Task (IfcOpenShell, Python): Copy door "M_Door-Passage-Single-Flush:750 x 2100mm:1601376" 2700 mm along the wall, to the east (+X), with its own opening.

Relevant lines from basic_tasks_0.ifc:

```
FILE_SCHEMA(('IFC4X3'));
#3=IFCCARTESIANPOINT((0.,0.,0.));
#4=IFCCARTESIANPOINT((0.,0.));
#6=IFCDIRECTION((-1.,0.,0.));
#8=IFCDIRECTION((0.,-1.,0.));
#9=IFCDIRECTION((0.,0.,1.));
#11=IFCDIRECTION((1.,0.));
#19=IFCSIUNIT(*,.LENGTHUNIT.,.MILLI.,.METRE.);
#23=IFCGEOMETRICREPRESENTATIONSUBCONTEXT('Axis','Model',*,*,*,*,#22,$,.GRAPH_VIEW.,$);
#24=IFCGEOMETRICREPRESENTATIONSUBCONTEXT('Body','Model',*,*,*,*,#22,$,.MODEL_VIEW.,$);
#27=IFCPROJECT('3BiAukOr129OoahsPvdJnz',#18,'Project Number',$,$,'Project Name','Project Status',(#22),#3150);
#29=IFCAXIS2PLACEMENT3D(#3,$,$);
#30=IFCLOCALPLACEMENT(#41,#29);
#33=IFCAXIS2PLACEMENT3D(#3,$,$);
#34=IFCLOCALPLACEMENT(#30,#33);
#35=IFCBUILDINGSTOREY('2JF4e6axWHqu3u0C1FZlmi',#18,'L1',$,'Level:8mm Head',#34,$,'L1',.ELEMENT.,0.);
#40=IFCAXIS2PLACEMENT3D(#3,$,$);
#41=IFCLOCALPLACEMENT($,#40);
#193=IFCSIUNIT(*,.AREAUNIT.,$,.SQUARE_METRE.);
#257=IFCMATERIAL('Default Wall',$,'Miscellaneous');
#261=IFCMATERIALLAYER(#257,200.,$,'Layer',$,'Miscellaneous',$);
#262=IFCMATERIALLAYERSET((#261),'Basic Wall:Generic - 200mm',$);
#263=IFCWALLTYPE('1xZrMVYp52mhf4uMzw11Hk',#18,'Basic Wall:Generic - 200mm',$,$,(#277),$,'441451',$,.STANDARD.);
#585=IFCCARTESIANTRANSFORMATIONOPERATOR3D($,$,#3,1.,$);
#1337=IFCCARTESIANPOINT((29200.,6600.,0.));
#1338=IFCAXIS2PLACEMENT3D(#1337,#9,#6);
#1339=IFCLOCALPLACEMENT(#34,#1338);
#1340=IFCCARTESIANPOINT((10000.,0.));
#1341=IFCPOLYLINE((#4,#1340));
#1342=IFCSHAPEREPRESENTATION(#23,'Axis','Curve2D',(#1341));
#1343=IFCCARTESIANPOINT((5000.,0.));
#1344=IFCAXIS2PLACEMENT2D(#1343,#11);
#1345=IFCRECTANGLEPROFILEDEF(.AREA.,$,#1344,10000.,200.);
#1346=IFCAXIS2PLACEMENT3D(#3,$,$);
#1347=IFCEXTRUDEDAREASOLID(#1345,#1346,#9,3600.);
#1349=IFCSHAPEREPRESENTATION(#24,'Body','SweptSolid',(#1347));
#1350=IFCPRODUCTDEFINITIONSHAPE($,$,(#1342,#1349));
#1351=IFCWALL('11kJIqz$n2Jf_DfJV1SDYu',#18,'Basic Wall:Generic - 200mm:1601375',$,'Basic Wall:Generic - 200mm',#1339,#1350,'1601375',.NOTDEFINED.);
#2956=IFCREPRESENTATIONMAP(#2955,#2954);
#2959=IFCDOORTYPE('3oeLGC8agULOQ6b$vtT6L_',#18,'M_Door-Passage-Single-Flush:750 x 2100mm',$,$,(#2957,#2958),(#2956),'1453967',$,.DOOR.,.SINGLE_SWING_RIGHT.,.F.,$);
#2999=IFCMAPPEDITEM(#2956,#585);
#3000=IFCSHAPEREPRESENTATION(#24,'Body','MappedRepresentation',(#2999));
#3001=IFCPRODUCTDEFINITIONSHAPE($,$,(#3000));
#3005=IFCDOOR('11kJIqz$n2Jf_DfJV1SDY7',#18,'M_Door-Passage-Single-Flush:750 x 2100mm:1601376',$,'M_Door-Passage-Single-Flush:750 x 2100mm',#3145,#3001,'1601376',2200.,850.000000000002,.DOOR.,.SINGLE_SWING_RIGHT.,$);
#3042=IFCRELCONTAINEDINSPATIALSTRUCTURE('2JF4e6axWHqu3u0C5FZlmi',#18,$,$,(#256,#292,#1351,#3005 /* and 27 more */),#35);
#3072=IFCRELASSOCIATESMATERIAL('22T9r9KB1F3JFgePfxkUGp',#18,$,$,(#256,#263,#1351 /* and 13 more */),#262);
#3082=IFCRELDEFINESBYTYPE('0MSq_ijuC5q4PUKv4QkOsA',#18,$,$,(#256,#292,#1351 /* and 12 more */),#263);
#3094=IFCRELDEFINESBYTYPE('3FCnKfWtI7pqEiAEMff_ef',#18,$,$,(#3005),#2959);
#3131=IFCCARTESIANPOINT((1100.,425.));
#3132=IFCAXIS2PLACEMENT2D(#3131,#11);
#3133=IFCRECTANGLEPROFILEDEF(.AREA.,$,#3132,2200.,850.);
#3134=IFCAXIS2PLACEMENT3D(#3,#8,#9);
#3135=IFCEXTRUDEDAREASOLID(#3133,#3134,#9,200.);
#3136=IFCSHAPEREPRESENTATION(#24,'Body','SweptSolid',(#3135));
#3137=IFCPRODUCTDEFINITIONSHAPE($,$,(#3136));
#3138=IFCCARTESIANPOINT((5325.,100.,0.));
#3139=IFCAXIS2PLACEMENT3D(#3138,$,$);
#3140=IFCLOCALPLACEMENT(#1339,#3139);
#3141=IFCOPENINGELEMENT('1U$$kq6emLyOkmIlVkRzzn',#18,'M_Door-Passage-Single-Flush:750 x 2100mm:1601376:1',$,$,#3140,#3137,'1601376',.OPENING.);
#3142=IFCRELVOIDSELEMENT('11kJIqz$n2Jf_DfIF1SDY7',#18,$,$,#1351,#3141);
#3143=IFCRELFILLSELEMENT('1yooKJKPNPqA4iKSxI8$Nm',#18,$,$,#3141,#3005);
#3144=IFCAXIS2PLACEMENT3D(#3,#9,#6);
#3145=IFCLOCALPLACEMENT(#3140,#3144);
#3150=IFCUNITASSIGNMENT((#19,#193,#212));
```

```python
import ifcopenshell
import ifcopenshell.api.feature
import ifcopenshell.api.geometry
import ifcopenshell.api.root
import ifcopenshell.geom
import ifcopenshell.util.element
import ifcopenshell.util.placement
import ifcopenshell.util.shape
import ifcopenshell.util.unit

model = ifcopenshell.open("basic_tasks_0.ifc")
unit_scale = ifcopenshell.util.unit.calculate_unit_scale(model)
settings = ifcopenshell.geom.settings()


def volume(element):
    """Net volume in cubic metres, openings subtracted."""
    shape = ifcopenshell.geom.create_shape(settings, element)
    return ifcopenshell.util.shape.get_volume(shape.geometry)


def reuse_history(source, copy):
    """copy_class also copies each property set's owner history, people and application; keep the originals."""
    for rel in copy.IsDefinedBy:
        if rel.is_a("IfcRelDefinesByProperties") and (history := rel.RelatingPropertyDefinition.OwnerHistory):
            rel.RelatingPropertyDefinition.OwnerHistory = source.OwnerHistory
            ifcopenshell.util.element.remove_deep2(model, history)


door = model.by_guid("11kJIqz$n2Jf_DfJV1SDY7")
opening = door.FillsVoids[0].RelatingOpeningElement
wall = opening.VoidsElements[0].RelatingBuildingElement
before = volume(wall)
shift = ifcopenshell.util.placement.get_local_placement(wall.ObjectPlacement)[:3, 0] * -2.7 / unit_scale

# copy_class copies the void relationship, type, container and properties, but no geometry.
new_opening = ifcopenshell.api.root.copy_class(model, product=opening)
new_opening.Representation = ifcopenshell.util.element.copy_deep(
    model, opening.Representation, exclude=["IfcGeometricRepresentationContext", "IfcRepresentationMap"]
)
new_opening.Name = "M_Door-Passage-Single-Flush:750 x 2100mm"
new_opening.Tag = None
new_door = ifcopenshell.api.root.copy_class(model, product=door)
new_door.Representation = ifcopenshell.util.element.copy_deep(
    model, door.Representation, exclude=["IfcGeometricRepresentationContext", "IfcRepresentationMap"]
)
new_door.Name = "M_Door-Passage-Single-Flush:750 x 2100mm"
new_door.Tag = None
reuse_history(door, new_door)
ifcopenshell.api.feature.add_filling(model, opening=new_opening, element=new_door)

for old, new in ((opening, new_opening), (door, new_door)):
    matrix = ifcopenshell.util.placement.get_local_placement(old.ObjectPlacement)
    matrix[:3, 3] += shift
    ifcopenshell.api.geometry.edit_object_placement(model, product=new, matrix=matrix, is_si=False)

after = volume(wall)

print(f"wall volume {before:.3f} -> {after:.3f} m3")

model.write("basic_tasks_0_rev.ifc")
```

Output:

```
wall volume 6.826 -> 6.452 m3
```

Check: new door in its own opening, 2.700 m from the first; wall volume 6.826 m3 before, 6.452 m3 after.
